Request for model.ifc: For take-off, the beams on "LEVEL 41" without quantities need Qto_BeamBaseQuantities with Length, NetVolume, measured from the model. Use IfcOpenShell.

First a look at what the model holds.

```python
import ifcopenshell
import ifcopenshell.util.element
import ifcopenshell.util.unit

model = ifcopenshell.open("model.ifc")
print(model.schema)
for unit_type in ("LENGTHUNIT", "AREAUNIT", "VOLUMEUNIT"):
    print(unit_type, ifcopenshell.util.unit.calculate_unit_scale(model, unit_type))
storey = next(s for s in model.by_type("IfcBuildingStorey") if s.Name == "LEVEL 41")
beams = [e for e in ifcopenshell.util.element.get_decomposition(storey) if e.is_a("IfcBeam")]
for e in sorted(beams, key=lambda e: e.id()):
    print(e.id(), e.is_a(), e.Name, list(ifcopenshell.util.element.get_psets(e, qtos_only=True)), sep=" | ")
```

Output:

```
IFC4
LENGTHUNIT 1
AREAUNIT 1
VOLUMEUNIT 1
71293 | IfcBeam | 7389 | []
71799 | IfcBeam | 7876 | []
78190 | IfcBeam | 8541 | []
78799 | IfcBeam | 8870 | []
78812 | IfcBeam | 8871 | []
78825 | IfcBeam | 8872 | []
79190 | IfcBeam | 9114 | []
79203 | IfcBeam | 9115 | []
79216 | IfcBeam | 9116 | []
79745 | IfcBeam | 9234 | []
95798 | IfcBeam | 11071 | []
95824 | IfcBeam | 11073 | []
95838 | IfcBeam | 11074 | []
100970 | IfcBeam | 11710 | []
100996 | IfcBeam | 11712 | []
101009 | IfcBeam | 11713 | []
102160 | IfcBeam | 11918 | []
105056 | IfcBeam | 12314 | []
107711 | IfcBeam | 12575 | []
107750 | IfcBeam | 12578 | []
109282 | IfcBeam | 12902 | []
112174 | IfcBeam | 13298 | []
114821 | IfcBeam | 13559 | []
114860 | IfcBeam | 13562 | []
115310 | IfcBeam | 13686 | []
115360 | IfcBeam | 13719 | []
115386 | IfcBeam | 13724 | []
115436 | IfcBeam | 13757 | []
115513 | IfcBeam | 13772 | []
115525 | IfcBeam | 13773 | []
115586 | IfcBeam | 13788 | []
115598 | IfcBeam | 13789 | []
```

```python
import ifcopenshell
import ifcopenshell.api.pset
import ifcopenshell.geom
import ifcopenshell.util.element
import ifcopenshell.util.shape
import ifcopenshell.util.unit

model = ifcopenshell.open("model.ifc")
unit_scale = ifcopenshell.util.unit.calculate_unit_scale(model)
volume_scale = ifcopenshell.util.unit.calculate_unit_scale(model, "VOLUMEUNIT")
settings = ifcopenshell.geom.settings()

storey = next(s for s in model.by_type("IfcBuildingStorey") if s.Name == "LEVEL 41")
beams = [e for e in ifcopenshell.util.element.get_decomposition(storey) if e.is_a("IfcBeam")]

for e in sorted(beams, key=lambda e: e.id()):
    if ifcopenshell.util.element.get_psets(e, qtos_only=True, should_inherit=False):
        continue
    # Geometry comes back in metres, in the element's own axes.
    shape = ifcopenshell.geom.create_shape(settings, e)
    values = {
        "Length": ifcopenshell.util.shape.get_max_xyz(shape.geometry) / unit_scale,
        "NetVolume": ifcopenshell.util.shape.get_volume(shape.geometry) / volume_scale,
    }
    qto = ifcopenshell.api.pset.add_qto(model, product=e, name="Qto_BeamBaseQuantities")
    ifcopenshell.api.pset.edit_qto(model, qto=qto, properties=values)
    print(e.id(), {k: round(v, 3) for k, v in values.items()})

model.write("model_rev.ifc")
```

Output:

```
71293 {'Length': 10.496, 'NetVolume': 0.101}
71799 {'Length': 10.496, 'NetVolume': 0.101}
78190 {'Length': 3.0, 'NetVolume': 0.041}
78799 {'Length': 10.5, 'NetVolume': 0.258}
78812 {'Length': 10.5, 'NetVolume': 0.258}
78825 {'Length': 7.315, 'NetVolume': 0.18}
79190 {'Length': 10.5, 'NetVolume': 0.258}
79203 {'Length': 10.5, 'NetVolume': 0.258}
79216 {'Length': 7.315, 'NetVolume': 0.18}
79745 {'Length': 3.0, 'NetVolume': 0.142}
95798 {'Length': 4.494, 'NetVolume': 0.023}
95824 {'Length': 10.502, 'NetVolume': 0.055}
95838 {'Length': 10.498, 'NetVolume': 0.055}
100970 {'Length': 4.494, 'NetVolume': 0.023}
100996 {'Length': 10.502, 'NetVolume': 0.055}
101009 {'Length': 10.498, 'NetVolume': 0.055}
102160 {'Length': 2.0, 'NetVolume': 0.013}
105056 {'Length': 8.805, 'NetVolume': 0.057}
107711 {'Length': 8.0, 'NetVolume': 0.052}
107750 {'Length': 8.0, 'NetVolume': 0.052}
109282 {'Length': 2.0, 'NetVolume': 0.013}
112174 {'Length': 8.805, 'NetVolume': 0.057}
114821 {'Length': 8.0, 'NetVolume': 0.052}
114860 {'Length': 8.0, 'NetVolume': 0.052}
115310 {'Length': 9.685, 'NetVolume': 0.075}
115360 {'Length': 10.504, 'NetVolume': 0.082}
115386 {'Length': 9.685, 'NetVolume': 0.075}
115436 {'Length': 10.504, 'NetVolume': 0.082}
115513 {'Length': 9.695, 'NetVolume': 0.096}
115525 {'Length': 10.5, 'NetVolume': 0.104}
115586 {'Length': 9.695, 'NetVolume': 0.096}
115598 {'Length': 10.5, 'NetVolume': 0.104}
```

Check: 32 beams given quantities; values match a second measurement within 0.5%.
